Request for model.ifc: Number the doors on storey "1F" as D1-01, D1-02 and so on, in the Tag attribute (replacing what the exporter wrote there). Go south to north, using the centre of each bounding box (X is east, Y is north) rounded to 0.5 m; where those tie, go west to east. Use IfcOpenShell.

First a look at what the model holds.

```python
import ifcopenshell
import ifcopenshell.util.element
import ifcopenshell.util.placement

model = ifcopenshell.open("model.ifc")
print(model.schema)
storey = next(s for s in model.by_type("IfcBuildingStorey") if s.Name == "1F")
doors = [e for e in ifcopenshell.util.element.get_decomposition(storey) if e.is_a("IfcDoor")]
for e in sorted(doors, key=lambda e: e.id()):
    origin = ifcopenshell.util.placement.get_local_placement(e.ObjectPlacement)[:3, 3]
    print(e.id(), e.Tag, e.Name, origin.round(2) + 0.0, sep=" | ")
```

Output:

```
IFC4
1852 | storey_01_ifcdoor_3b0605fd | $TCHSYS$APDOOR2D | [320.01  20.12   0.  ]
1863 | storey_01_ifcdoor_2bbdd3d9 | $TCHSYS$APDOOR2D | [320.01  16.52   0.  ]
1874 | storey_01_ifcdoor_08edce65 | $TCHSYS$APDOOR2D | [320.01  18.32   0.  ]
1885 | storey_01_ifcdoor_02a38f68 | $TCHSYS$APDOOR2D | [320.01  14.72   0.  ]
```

```python
import ifcopenshell
import ifcopenshell.geom
import ifcopenshell.util.element
import ifcopenshell.util.shape

model = ifcopenshell.open("model.ifc")
settings = ifcopenshell.geom.settings()
settings.set("use-world-coords", True)


def centre(element):
    shape = ifcopenshell.geom.create_shape(settings, element)
    return ifcopenshell.util.shape.get_bbox_centroid(shape.geometry)


storey = next(s for s in model.by_type("IfcBuildingStorey") if s.Name == "1F")
doors = [e for e in ifcopenshell.util.element.get_decomposition(storey) if e.is_a("IfcDoor")]

# Insertion points can sit at a corner or the storey origin, so sort by the geometry (in metres).
centres = {e: centre(e) for e in doors}
doors.sort(key=lambda e: (round(centres[e][1] / 0.5), centres[e][0]))

for i, e in enumerate(doors, start=1):
    number = f"D1-{i:02d}"
    e.Tag = number
    print(e.id(), number)

model.write("model_updated.ifc")
```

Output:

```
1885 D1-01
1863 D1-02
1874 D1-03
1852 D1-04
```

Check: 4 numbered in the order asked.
